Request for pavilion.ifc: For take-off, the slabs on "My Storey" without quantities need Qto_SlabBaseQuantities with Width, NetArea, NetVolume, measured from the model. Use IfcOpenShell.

First a look at what the model holds.

```python
import ifcopenshell
import ifcopenshell.util.element
import ifcopenshell.util.unit

model = ifcopenshell.open("pavilion.ifc")
print(model.schema)
for unit_type in ("LENGTHUNIT", "AREAUNIT", "VOLUMEUNIT"):
    print(unit_type, ifcopenshell.util.unit.calculate_unit_scale(model, unit_type))
storey = next(s for s in model.by_type("IfcBuildingStorey") if s.Name == "My Storey")
slabs = [e for e in ifcopenshell.util.element.get_decomposition(storey) if e.is_a("IfcSlab")]
for e in sorted(slabs, key=lambda e: e.id()):
    print(e.id(), e.is_a(), e.Name, list(ifcopenshell.util.element.get_psets(e, qtos_only=True)), sep=" | ")
```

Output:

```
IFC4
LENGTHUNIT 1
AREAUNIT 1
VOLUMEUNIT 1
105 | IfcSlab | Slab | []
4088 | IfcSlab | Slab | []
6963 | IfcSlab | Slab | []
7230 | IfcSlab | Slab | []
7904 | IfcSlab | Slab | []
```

```python
import ifcopenshell
import ifcopenshell.api.pset
import ifcopenshell.geom
import ifcopenshell.util.element
import ifcopenshell.util.shape
import ifcopenshell.util.unit

model = ifcopenshell.open("pavilion.ifc")
unit_scale = ifcopenshell.util.unit.calculate_unit_scale(model)
area_scale = ifcopenshell.util.unit.calculate_unit_scale(model, "AREAUNIT")
volume_scale = ifcopenshell.util.unit.calculate_unit_scale(model, "VOLUMEUNIT")
settings = ifcopenshell.geom.settings()

storey = next(s for s in model.by_type("IfcBuildingStorey") if s.Name == "My Storey")
slabs = [e for e in ifcopenshell.util.element.get_decomposition(storey) if e.is_a("IfcSlab")]

for e in sorted(slabs, key=lambda e: e.id()):
    if ifcopenshell.util.element.get_psets(e, qtos_only=True, should_inherit=False):
        continue
    # Geometry comes back in metres, in the element's own axes.
    shape = ifcopenshell.geom.create_shape(settings, e)
    values = {
        "Width": ifcopenshell.util.shape.get_z(shape.geometry) / unit_scale,
        "NetArea": ifcopenshell.util.shape.get_footprint_area(shape.geometry) / area_scale,
        "NetVolume": ifcopenshell.util.shape.get_volume(shape.geometry) / volume_scale,
    }
    qto = ifcopenshell.api.pset.add_qto(model, product=e, name="Qto_SlabBaseQuantities")
    ifcopenshell.api.pset.edit_qto(model, qto=qto, properties=values)
    print(e.id(), {k: round(v, 3) for k, v in values.items()})

model.write("pavilion_updated.ifc")
```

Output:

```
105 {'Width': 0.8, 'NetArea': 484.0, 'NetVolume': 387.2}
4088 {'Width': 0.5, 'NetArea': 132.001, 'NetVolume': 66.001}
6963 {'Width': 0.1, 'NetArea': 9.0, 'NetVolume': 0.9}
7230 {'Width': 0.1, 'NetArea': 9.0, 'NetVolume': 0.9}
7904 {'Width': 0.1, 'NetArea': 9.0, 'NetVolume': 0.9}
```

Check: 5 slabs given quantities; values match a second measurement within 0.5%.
